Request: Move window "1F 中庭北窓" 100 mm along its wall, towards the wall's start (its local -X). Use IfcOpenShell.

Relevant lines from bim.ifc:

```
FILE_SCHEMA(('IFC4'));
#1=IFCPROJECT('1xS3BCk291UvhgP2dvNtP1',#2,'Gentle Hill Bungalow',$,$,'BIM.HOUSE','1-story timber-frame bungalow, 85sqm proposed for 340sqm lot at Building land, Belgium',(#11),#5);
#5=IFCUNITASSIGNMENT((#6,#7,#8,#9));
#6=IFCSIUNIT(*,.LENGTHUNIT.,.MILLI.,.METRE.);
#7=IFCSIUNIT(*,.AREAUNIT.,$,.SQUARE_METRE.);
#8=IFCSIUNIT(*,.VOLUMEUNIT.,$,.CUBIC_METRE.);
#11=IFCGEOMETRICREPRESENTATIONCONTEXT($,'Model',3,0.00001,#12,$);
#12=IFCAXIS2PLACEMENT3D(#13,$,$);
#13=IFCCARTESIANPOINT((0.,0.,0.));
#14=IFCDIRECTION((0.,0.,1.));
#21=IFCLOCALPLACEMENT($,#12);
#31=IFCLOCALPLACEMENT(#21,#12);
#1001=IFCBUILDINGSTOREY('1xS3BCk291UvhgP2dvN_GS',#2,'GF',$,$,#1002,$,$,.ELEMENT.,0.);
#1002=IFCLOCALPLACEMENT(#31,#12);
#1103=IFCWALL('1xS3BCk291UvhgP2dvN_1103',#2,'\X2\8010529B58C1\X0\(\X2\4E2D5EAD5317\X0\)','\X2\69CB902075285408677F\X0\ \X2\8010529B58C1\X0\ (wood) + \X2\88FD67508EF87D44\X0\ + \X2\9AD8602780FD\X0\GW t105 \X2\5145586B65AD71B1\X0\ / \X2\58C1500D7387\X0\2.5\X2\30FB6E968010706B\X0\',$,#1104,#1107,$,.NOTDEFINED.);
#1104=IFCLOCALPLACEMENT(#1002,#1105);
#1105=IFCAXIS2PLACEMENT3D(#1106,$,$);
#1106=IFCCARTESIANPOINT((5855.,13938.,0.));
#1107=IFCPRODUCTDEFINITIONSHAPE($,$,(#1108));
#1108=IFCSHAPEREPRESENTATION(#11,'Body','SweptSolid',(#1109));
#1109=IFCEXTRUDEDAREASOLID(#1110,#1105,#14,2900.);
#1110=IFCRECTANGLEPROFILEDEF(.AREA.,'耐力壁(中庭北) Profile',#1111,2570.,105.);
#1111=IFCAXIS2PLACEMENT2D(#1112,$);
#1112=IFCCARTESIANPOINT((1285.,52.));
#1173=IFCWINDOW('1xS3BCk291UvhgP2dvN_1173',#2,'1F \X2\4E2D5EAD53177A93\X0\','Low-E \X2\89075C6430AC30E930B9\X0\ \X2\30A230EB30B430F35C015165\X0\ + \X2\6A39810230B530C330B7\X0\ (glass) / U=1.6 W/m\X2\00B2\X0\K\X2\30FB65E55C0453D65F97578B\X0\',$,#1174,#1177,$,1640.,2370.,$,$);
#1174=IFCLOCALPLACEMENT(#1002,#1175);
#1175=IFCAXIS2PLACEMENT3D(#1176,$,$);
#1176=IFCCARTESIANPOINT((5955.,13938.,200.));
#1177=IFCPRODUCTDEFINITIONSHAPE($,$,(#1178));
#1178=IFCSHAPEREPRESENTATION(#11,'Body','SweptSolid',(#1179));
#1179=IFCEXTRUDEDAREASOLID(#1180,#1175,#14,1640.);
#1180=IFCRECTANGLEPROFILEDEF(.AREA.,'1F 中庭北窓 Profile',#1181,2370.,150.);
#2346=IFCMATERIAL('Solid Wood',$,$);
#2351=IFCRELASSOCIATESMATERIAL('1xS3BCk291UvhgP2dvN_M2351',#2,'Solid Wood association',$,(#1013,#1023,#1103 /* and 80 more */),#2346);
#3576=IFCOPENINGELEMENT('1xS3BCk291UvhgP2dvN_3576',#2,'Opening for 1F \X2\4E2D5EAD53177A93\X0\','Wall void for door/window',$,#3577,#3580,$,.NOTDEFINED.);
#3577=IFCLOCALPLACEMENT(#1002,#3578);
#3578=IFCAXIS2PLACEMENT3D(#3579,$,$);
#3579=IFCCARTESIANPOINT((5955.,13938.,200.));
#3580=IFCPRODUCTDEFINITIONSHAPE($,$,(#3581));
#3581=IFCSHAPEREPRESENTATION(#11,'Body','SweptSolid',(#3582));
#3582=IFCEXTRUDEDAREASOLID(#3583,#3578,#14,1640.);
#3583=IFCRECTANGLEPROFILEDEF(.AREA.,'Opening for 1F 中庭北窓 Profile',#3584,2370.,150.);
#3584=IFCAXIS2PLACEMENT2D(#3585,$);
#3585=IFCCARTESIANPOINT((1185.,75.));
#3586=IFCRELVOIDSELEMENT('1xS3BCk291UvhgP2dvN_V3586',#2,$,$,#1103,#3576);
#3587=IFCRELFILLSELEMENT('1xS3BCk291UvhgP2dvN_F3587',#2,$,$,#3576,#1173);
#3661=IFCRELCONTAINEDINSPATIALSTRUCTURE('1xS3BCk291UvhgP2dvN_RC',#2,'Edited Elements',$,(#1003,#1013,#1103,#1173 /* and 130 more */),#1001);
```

```python
import ifcopenshell
import ifcopenshell.api.geometry
import ifcopenshell.util.placement
import ifcopenshell.util.unit

model = ifcopenshell.open("bim.ifc")
unit_scale = ifcopenshell.util.unit.calculate_unit_scale(model)

window = model.by_id(1173)
opening = window.FillsVoids[0].RelatingOpeningElement
wall = opening.VoidsElements[0].RelatingBuildingElement

wall_matrix = ifcopenshell.util.placement.get_local_placement(wall.ObjectPlacement)
shift = wall_matrix[:3, 0] * -0.1 / unit_scale
before = ifcopenshell.util.placement.get_local_placement(window.ObjectPlacement)[:3, 3].copy()

# The window is not placed relative to its opening, so move both.
for product in (opening, window):
    matrix = ifcopenshell.util.placement.get_local_placement(product.ObjectPlacement)
    matrix[:3, 3] += shift
    ifcopenshell.api.geometry.edit_object_placement(model, product=product, matrix=matrix, is_si=False)

after = ifcopenshell.util.placement.get_local_placement(window.ObjectPlacement)[:3, 3]
print("window moved by", (after - before).round(3) + 0.0)

model.write("bim-out.ifc")
```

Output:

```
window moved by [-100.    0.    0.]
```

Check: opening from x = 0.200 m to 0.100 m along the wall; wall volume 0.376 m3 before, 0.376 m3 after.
